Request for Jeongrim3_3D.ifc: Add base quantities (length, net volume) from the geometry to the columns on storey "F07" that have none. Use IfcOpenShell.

First a look at what the model holds.

```python
import ifcopenshell
import ifcopenshell.util.element
import ifcopenshell.util.unit

model = ifcopenshell.open("Jeongrim3_3D.ifc")
print(model.schema)
for unit_type in ("LENGTHUNIT", "AREAUNIT", "VOLUMEUNIT"):
    print(unit_type, ifcopenshell.util.unit.calculate_unit_scale(model, unit_type))
storey = next(s for s in model.by_type("IfcBuildingStorey") if s.Name == "F07")
columns = [e for e in ifcopenshell.util.element.get_decomposition(storey) if e.is_a("IfcColumn")]
for e in sorted(columns, key=lambda e: e.id()):
    print(e.id(), e.is_a(), e.Name, list(ifcopenshell.util.element.get_psets(e, qtos_only=True)), sep=" | ")
```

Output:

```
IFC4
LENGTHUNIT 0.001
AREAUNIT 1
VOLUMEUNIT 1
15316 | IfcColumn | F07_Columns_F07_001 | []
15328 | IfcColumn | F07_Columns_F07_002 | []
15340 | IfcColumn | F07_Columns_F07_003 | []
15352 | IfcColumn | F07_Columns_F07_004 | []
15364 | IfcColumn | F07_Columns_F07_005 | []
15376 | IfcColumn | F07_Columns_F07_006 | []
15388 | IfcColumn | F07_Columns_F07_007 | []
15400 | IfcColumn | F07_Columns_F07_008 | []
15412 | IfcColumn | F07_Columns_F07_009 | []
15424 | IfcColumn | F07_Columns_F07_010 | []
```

```python
import ifcopenshell
import ifcopenshell.api.pset
import ifcopenshell.geom
import ifcopenshell.util.element
import ifcopenshell.util.shape
import ifcopenshell.util.unit

model = ifcopenshell.open("Jeongrim3_3D.ifc")
unit_scale = ifcopenshell.util.unit.calculate_unit_scale(model)
volume_scale = ifcopenshell.util.unit.calculate_unit_scale(model, "VOLUMEUNIT")
settings = ifcopenshell.geom.settings()

storey = next(s for s in model.by_type("IfcBuildingStorey") if s.Name == "F07")
columns = [e for e in ifcopenshell.util.element.get_decomposition(storey) if e.is_a("IfcColumn")]

for e in sorted(columns, key=lambda e: e.id()):
    if ifcopenshell.util.element.get_psets(e, qtos_only=True, should_inherit=False):
        continue
    # Geometry comes back in metres, in the element's own axes.
    shape = ifcopenshell.geom.create_shape(settings, e)
    values = {
        "Length": ifcopenshell.util.shape.get_z(shape.geometry) / unit_scale,
        "NetVolume": ifcopenshell.util.shape.get_volume(shape.geometry) / volume_scale,
    }
    qto = ifcopenshell.api.pset.add_qto(model, product=e, name="Qto_ColumnBaseQuantities")
    ifcopenshell.api.pset.edit_qto(model, qto=qto, properties=values)
    print(e.id(), {k: round(v, 3) for k, v in values.items()})

model.write("Jeongrim3_3D_v2.ifc")
```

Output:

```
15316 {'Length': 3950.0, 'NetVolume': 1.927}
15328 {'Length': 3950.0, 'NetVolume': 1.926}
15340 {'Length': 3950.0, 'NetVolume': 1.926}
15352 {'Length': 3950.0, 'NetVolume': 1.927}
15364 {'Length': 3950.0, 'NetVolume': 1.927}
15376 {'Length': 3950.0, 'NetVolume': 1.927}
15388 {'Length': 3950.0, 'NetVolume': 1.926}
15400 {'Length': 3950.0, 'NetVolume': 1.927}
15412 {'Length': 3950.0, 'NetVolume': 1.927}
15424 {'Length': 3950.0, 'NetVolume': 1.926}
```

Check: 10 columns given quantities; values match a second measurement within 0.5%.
